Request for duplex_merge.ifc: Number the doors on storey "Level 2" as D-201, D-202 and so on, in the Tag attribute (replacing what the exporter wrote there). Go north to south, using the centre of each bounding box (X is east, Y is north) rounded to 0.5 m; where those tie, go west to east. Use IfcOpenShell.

First a look at what the model holds.

```python
import ifcopenshell
import ifcopenshell.util.element
import ifcopenshell.util.placement

model = ifcopenshell.open("duplex_merge.ifc")
print(model.schema)
storey = next(s for s in model.by_type("IfcBuildingStorey") if s.Name == "Level 2")
doors = [e for e in ifcopenshell.util.element.get_decomposition(storey) if e.is_a("IfcDoor")]
for e in sorted(doors, key=lambda e: e.id()):
    origin = ifcopenshell.util.placement.get_local_placement(e.ObjectPlacement)[:3, 3]
    print(e.id(), e.Tag, e.Name, origin.round(2) + 0.0, sep=" | ")
```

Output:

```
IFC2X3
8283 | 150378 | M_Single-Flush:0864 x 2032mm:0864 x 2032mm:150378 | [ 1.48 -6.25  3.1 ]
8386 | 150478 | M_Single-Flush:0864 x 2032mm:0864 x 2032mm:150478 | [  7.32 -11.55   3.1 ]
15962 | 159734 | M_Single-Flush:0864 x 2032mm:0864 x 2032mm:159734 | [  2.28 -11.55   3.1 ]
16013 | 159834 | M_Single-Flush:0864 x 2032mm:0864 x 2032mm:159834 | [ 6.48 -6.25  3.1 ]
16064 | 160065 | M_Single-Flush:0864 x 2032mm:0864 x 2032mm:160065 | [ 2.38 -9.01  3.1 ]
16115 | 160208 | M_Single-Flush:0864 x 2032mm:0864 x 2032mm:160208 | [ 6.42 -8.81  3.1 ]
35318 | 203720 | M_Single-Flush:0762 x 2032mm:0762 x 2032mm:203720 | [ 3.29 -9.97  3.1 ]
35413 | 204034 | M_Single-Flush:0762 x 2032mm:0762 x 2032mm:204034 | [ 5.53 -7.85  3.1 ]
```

```python
import ifcopenshell
import ifcopenshell.geom
import ifcopenshell.util.element
import ifcopenshell.util.shape

model = ifcopenshell.open("duplex_merge.ifc")
settings = ifcopenshell.geom.settings()
settings.set("use-world-coords", True)


def centre(element):
    shape = ifcopenshell.geom.create_shape(settings, element)
    return ifcopenshell.util.shape.get_bbox_centroid(shape.geometry)


storey = next(s for s in model.by_type("IfcBuildingStorey") if s.Name == "Level 2")
doors = [e for e in ifcopenshell.util.element.get_decomposition(storey) if e.is_a("IfcDoor")]

# Insertion points can sit at a corner or the storey origin, so sort by the geometry (in metres).
centres = {e: centre(e) for e in doors}
doors.sort(key=lambda e: (-round(centres[e][1] / 0.5), centres[e][0]))

for i, e in enumerate(doors, start=1):
    number = f"D-2{i:02d}"
    e.Tag = number
    print(e.id(), number)

model.write("duplex_merge_edited.ifc")
```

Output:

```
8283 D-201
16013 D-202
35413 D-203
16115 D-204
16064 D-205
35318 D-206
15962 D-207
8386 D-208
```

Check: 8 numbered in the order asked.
